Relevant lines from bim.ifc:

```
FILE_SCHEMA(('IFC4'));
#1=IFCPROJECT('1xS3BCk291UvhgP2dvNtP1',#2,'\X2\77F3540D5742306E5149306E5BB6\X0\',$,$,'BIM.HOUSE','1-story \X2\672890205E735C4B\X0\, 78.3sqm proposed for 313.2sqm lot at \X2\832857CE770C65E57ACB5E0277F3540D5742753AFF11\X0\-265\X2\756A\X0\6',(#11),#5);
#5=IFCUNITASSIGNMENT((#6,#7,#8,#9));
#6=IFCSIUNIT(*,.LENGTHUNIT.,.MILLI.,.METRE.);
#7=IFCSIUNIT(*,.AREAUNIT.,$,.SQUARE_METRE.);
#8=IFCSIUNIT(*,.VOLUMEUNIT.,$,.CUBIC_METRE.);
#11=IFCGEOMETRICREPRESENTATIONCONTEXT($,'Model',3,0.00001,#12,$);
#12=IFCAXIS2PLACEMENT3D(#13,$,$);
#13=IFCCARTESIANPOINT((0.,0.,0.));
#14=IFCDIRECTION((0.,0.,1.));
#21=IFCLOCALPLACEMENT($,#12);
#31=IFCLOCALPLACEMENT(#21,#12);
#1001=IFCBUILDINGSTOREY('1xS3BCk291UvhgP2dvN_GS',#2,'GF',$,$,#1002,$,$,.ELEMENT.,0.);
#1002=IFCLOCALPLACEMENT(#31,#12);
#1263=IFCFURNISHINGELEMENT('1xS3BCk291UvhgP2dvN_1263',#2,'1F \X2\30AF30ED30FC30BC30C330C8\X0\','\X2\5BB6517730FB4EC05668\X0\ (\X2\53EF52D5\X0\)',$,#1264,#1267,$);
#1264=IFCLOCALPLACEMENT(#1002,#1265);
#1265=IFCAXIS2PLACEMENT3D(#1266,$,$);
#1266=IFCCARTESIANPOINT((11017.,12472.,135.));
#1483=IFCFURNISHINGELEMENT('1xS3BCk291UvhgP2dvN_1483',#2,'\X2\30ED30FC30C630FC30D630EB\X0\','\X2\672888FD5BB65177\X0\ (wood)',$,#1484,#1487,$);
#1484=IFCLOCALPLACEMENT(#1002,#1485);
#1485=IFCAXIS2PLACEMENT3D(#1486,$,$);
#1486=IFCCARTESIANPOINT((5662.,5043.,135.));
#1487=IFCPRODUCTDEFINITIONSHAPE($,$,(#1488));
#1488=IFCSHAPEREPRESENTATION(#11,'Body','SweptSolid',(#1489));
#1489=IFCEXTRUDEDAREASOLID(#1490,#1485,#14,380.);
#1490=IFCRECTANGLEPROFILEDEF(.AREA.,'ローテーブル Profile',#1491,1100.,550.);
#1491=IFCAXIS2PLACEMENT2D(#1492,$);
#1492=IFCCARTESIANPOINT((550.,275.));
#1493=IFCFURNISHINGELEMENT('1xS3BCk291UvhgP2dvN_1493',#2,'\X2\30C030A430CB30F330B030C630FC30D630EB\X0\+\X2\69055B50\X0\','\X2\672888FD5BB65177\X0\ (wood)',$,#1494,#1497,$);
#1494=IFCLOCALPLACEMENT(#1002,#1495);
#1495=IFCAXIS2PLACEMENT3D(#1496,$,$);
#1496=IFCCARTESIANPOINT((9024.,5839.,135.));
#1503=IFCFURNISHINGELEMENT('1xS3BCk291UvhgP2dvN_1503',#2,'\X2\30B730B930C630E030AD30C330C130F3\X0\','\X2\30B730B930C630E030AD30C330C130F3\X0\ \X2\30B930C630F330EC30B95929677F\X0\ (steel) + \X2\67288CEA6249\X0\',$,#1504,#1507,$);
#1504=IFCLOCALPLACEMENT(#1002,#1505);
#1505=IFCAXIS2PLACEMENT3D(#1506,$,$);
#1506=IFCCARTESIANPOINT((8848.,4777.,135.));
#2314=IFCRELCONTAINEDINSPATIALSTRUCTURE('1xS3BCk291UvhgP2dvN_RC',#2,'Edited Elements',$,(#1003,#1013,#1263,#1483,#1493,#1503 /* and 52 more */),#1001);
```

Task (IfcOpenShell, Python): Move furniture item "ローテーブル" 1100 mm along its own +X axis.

```python
import ifcopenshell
import ifcopenshell.api.geometry
import ifcopenshell.util.placement
import ifcopenshell.util.unit

model = ifcopenshell.open("bim.ifc")
unit_scale = ifcopenshell.util.unit.calculate_unit_scale(model)

item = model.by_id(1483)
matrix = ifcopenshell.util.placement.get_local_placement(item.ObjectPlacement)
matrix[:3, 3] += matrix[:3, 0] * 1.1 / unit_scale
ifcopenshell.api.geometry.edit_object_placement(model, product=item, matrix=matrix, is_si=False)

print(ifcopenshell.util.placement.get_local_placement(item.ObjectPlacement).round(3) + 0.0)

model.write("bim_v2.ifc")
```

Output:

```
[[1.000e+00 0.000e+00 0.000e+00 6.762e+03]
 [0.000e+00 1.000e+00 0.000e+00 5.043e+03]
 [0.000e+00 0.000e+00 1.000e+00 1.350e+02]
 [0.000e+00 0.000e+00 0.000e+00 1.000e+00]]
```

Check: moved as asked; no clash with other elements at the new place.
